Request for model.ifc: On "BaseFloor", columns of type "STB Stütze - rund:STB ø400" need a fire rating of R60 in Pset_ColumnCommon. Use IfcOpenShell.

First a look at what the model holds.

```python
import ifcopenshell
import ifcopenshell.util.element

model = ifcopenshell.open("model.ifc")
print(model.schema)
storey = next(s for s in model.by_type("IfcBuildingStorey") if s.Name == "BaseFloor")
columns = [e for e in ifcopenshell.util.element.get_decomposition(storey) if e.is_a("IfcColumn")]
seen = {}
for e in columns:
    element_type = ifcopenshell.util.element.get_type(e)
    key = (element_type.Name if element_type != e and element_type else None, ifcopenshell.util.element.get_pset(e, "Pset_ColumnCommon", "FireRating"))
    seen[key] = seen.get(key, 0) + 1
for (name, value), count in sorted(seen.items(), key=str):
    print(count, "x", name, "|", value)
```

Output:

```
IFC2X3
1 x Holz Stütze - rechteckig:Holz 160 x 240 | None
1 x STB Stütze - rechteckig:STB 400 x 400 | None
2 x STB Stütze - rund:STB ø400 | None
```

```python
import ifcopenshell
import ifcopenshell.api.pset
import ifcopenshell.util.element

model = ifcopenshell.open("model.ifc")

storey = next(s for s in model.by_type("IfcBuildingStorey") if s.Name == "BaseFloor")
columns = [e for e in ifcopenshell.util.element.get_decomposition(storey) if e.is_a("IfcColumn")]

count = 0
for e in columns:
    element_type = ifcopenshell.util.element.get_type(e)
    if element_type in (None, e) or element_type.Name != "STB Stütze - rund:STB ø400":
        continue
    # add_pset returns the element's existing set when there is one.
    pset = ifcopenshell.api.pset.add_pset(model, product=e, name="Pset_ColumnCommon")
    ifcopenshell.api.pset.edit_pset(model, pset=pset, properties={"FireRating": "R60"})
    count += 1

print(count, "columns updated")

model.write("model_edited.ifc")
```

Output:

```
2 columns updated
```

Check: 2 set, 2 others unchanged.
